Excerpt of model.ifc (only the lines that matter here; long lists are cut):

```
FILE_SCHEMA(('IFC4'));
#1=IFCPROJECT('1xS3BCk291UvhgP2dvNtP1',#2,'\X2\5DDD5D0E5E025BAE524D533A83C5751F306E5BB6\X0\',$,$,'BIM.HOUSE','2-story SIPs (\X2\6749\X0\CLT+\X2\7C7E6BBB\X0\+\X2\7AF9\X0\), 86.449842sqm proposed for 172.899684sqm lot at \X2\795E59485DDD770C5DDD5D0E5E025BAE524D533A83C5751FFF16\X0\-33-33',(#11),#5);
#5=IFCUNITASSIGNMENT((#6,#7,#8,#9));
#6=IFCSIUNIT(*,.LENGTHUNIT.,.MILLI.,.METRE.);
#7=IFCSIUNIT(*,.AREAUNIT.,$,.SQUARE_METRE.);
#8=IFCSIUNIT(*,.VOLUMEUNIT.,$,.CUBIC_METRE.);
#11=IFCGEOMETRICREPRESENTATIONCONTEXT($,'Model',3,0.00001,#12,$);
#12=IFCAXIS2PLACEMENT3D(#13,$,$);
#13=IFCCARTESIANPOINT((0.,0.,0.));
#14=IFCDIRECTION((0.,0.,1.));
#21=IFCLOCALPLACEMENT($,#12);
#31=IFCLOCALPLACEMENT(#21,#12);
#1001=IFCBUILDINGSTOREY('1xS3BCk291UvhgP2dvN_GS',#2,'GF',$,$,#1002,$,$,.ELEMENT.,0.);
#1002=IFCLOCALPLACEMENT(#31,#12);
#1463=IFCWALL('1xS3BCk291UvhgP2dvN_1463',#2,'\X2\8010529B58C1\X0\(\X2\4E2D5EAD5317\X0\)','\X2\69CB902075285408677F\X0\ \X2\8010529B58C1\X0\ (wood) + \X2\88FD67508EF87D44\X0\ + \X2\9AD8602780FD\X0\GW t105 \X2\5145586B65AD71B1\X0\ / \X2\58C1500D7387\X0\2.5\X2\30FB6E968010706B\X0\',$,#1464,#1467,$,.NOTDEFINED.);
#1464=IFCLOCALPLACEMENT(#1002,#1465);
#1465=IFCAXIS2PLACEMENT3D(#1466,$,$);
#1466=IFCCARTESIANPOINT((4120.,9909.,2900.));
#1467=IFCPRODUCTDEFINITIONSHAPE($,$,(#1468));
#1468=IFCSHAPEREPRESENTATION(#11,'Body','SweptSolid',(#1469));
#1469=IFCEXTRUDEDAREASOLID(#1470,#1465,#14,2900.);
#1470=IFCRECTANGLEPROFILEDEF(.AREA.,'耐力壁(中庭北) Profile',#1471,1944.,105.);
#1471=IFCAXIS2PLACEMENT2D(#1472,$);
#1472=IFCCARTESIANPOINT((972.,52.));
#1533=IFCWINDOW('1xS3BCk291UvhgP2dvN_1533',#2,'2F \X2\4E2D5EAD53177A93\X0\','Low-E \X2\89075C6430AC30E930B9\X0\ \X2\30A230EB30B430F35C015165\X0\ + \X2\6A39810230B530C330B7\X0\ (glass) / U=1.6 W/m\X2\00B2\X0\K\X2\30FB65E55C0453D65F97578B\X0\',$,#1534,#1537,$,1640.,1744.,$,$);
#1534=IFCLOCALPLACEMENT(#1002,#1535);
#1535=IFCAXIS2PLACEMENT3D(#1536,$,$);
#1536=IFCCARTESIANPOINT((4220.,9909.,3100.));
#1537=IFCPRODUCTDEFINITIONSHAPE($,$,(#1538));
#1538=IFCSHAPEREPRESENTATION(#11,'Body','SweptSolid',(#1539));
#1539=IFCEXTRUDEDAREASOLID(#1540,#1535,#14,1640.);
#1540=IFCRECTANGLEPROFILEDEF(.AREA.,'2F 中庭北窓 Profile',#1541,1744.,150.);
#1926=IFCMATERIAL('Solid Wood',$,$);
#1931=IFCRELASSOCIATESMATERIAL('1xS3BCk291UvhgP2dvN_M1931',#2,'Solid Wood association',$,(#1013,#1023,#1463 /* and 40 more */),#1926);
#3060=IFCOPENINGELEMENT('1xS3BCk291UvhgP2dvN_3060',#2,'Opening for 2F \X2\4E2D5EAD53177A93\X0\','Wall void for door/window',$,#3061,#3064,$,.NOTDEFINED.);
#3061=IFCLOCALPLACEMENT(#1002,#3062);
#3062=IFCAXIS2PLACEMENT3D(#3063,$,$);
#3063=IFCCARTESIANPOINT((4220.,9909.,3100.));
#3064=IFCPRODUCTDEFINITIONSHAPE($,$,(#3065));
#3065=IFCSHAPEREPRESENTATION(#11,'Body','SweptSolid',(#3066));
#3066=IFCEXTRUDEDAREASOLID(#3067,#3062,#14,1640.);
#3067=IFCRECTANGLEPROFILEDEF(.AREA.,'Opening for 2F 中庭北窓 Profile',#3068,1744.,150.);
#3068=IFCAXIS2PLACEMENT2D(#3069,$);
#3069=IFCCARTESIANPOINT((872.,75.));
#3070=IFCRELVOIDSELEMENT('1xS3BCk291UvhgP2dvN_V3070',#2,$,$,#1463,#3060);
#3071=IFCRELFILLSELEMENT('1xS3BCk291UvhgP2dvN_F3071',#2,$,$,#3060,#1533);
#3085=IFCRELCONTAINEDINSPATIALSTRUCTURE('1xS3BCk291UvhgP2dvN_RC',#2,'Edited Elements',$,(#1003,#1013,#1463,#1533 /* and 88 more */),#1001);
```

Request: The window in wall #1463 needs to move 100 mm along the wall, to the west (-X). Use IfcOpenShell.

```python
import ifcopenshell
import ifcopenshell.api.geometry
import ifcopenshell.util.placement
import ifcopenshell.util.unit

model = ifcopenshell.open("model.ifc")
unit_scale = ifcopenshell.util.unit.calculate_unit_scale(model)

window = model.by_id(1533)
opening = window.FillsVoids[0].RelatingOpeningElement
wall = opening.VoidsElements[0].RelatingBuildingElement

wall_matrix = ifcopenshell.util.placement.get_local_placement(wall.ObjectPlacement)
shift = wall_matrix[:3, 0] * -0.1 / unit_scale
before = ifcopenshell.util.placement.get_local_placement(window.ObjectPlacement)[:3, 3].copy()

# The window is not placed relative to its opening, so move both.
for product in (opening, window):
    matrix = ifcopenshell.util.placement.get_local_placement(product.ObjectPlacement)
    matrix[:3, 3] += shift
    ifcopenshell.api.geometry.edit_object_placement(model, product=product, matrix=matrix, is_si=False)

after = ifcopenshell.util.placement.get_local_placement(window.ObjectPlacement)[:3, 3]
print("window moved by", (after - before).round(3) + 0.0)

model.write("model_edited.ifc")
```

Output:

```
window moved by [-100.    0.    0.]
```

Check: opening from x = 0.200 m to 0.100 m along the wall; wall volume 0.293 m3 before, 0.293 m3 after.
